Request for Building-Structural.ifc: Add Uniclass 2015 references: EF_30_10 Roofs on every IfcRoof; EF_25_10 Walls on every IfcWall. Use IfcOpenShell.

First a look at what the model holds.

```python
import ifcopenshell

model = ifcopenshell.open("Building-Structural.ifc")
print(model.schema)
print("classifications:", [c.Name for c in model.by_type("IfcClassification")])
for ifc_class in ("IfcDoor", "IfcRoof", "IfcStair", "IfcWall", "IfcWindow"):
    print(ifc_class, len(model.by_type(ifc_class)))
```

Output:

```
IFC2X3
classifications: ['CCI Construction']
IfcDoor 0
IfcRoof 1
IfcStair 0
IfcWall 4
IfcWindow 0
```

```python
import ifcopenshell
import ifcopenshell.api.classification

model = ifcopenshell.open("Building-Structural.ifc")

# IFC2X3 requires Source and Edition and has no link from the project to the system.
system = model.create_entity("IfcClassification", Source="NBS", Edition="2015", Name="Uniclass 2015")

codes = {
    "IfcRoof": ("EF_30_10", "Roofs"),
    "IfcWall": ("EF_25_10", "Walls"),
}
for ifc_class, (code, name) in codes.items():
    products = model.by_type(ifc_class)
    ifcopenshell.api.classification.add_reference(
        model, products=products, classification=system, identification=code, name=name
    )
    print(code, len(products))

model.write("Building-Structural_updated.ifc")
```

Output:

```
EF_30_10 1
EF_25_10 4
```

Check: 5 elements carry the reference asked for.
